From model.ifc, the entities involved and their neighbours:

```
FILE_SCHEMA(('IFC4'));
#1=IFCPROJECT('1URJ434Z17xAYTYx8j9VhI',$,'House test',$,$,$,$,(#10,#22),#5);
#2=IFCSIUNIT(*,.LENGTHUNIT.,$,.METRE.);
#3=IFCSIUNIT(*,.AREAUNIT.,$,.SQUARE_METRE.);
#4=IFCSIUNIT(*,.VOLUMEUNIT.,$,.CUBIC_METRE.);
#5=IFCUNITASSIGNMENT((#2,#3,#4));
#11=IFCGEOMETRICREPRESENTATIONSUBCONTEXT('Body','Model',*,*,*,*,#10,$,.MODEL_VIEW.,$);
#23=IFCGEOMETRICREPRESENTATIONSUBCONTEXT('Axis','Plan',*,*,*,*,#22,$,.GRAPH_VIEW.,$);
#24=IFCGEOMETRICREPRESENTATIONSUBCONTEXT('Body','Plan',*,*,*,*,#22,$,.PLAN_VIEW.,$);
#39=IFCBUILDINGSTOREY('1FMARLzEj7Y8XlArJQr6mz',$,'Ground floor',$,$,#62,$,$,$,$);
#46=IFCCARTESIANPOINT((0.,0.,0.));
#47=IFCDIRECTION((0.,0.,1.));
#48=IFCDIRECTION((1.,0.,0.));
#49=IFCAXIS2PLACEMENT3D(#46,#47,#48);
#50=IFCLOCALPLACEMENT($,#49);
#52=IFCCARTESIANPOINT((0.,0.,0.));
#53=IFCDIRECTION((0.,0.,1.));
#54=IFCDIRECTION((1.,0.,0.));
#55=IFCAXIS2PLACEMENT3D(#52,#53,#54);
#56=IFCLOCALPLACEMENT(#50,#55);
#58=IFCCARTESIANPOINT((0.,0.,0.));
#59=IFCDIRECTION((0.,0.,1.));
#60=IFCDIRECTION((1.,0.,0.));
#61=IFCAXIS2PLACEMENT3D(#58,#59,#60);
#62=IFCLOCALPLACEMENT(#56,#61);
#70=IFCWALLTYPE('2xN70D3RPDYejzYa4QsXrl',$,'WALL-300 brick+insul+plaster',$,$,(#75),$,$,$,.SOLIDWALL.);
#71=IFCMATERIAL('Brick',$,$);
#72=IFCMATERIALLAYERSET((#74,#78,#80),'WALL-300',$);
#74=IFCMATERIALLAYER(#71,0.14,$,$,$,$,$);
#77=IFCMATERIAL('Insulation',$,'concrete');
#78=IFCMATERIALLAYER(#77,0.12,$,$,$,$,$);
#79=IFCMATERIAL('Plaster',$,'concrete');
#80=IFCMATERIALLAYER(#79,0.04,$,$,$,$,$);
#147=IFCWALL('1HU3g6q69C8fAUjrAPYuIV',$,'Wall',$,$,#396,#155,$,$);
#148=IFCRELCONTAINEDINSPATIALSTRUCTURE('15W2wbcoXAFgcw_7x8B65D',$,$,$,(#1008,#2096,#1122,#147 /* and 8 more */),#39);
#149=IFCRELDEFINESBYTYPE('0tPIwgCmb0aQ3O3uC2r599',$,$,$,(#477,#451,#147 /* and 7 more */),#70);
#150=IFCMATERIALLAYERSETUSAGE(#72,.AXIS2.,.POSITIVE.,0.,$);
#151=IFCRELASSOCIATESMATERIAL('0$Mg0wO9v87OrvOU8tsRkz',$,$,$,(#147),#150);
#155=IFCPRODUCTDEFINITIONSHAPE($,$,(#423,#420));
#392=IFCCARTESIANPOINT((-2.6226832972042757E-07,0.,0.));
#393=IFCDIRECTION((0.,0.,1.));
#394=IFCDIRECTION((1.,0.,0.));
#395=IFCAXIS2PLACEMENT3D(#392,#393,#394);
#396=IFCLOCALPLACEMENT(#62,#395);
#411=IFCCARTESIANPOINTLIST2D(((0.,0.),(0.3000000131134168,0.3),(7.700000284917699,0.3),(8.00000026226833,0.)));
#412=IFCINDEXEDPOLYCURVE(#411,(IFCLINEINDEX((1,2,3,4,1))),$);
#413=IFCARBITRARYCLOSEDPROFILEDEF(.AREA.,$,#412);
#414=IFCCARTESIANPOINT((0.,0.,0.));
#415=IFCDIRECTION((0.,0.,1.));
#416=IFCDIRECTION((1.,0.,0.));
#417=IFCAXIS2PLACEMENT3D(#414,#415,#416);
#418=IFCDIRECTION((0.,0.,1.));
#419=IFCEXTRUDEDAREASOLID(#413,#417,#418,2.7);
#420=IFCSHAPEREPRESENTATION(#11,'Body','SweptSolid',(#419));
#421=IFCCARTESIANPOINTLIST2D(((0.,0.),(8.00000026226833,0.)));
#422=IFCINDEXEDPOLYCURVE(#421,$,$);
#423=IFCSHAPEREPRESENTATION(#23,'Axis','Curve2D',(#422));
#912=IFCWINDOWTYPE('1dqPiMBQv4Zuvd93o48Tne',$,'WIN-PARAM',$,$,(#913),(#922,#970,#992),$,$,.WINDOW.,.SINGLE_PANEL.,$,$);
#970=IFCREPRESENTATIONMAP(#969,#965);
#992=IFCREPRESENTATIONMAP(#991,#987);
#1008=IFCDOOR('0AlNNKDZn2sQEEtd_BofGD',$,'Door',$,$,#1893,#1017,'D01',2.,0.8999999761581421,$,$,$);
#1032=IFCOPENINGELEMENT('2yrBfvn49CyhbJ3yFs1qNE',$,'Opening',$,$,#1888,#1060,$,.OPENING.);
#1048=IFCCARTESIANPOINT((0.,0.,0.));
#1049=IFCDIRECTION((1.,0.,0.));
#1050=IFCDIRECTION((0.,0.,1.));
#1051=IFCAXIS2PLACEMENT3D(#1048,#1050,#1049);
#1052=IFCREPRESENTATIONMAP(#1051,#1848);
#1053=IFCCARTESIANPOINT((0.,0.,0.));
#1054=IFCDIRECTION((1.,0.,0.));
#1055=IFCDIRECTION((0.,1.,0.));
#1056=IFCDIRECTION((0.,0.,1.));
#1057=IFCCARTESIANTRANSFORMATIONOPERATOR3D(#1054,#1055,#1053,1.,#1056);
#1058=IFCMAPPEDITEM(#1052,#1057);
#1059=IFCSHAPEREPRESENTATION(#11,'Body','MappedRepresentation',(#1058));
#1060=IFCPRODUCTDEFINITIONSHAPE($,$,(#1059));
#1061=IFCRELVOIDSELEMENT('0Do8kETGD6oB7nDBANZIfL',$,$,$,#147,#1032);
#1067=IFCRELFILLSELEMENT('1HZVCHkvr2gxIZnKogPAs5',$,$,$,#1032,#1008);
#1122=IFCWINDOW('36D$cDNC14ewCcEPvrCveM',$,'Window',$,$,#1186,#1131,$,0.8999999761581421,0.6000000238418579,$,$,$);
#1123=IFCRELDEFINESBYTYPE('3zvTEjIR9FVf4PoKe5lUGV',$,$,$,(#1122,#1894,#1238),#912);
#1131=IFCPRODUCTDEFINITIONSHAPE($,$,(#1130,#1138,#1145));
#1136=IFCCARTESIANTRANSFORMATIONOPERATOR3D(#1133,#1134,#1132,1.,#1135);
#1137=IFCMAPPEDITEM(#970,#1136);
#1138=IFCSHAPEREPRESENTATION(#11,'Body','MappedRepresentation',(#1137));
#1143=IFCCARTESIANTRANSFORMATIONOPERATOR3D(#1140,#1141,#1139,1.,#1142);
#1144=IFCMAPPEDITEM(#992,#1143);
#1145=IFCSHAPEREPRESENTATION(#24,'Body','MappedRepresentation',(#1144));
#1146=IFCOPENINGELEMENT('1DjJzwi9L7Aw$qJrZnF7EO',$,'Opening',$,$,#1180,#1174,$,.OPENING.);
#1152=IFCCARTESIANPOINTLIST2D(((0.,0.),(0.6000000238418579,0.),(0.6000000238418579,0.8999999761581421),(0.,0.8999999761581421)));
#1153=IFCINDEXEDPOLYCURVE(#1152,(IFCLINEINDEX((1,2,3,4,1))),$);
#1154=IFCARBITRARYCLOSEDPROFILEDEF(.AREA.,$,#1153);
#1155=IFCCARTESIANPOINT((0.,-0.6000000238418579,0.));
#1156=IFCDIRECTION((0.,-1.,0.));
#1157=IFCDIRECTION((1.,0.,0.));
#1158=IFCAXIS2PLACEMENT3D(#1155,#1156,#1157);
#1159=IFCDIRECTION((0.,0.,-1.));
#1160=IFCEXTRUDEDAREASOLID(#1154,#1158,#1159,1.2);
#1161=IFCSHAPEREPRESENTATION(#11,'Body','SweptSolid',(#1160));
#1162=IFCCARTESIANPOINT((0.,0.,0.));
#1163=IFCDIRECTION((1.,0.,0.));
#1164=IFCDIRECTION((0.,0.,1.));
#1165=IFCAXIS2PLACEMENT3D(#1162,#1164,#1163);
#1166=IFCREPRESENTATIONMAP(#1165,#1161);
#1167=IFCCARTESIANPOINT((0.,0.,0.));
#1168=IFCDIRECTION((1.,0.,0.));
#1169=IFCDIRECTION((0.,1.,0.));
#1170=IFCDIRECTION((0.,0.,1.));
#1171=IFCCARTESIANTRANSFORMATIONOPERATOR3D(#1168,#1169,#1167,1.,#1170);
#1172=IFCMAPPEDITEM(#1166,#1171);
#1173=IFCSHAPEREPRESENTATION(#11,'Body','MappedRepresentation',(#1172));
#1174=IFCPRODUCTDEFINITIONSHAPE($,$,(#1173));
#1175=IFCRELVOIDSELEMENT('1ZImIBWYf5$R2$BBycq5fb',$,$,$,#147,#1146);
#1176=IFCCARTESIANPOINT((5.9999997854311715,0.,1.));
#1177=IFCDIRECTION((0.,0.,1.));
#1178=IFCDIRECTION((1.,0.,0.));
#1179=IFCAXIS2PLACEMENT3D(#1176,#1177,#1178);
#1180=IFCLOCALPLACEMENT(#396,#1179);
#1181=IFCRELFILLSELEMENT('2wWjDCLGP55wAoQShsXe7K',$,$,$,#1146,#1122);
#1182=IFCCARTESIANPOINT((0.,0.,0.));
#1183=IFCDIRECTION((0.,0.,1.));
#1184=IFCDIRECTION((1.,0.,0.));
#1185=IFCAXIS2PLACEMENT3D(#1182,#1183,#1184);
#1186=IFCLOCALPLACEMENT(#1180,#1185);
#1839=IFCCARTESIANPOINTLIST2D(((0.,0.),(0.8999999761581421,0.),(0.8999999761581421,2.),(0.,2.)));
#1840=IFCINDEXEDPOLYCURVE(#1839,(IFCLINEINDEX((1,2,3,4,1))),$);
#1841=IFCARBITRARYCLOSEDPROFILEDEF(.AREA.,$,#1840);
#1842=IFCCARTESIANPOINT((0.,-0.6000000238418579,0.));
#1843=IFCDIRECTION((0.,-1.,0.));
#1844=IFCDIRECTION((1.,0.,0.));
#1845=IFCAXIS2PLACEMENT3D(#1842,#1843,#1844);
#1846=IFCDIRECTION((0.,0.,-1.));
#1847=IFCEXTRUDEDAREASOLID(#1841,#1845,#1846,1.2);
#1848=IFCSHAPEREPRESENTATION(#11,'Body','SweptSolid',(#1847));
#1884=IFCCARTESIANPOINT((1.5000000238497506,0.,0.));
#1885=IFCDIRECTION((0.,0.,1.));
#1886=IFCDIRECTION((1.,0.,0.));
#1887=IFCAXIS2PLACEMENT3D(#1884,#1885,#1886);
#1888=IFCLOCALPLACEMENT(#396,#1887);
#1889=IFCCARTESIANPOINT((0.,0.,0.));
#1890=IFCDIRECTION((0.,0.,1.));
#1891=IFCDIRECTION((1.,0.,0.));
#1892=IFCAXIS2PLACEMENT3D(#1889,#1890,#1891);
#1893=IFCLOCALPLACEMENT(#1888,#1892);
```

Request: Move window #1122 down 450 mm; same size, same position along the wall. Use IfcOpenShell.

```python
import numpy as np
import ifcopenshell
import ifcopenshell.api.geometry
import ifcopenshell.util.placement
import ifcopenshell.util.unit

model = ifcopenshell.open("model.ifc")
unit_scale = ifcopenshell.util.unit.calculate_unit_scale(model)

window = model.by_guid("36D$cDNC14ewCcEPvrCveM")
opening = window.FillsVoids[0].RelatingOpeningElement
dz = -0.45

shift = np.array([0.0, 0.0, dz])
# The window is placed relative to its opening, so it follows when the opening moves.
matrix = ifcopenshell.util.placement.get_local_placement(opening.ObjectPlacement)
matrix[:3, 3] += shift
ifcopenshell.api.geometry.edit_object_placement(
    model, product=opening, matrix=matrix, is_si=False, should_transform_children=True
)

print(f"moved by {dz * unit_scale:+.3f} m")

model.write("model_edited.ifc")
```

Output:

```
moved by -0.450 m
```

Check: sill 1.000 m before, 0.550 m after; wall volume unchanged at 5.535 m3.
